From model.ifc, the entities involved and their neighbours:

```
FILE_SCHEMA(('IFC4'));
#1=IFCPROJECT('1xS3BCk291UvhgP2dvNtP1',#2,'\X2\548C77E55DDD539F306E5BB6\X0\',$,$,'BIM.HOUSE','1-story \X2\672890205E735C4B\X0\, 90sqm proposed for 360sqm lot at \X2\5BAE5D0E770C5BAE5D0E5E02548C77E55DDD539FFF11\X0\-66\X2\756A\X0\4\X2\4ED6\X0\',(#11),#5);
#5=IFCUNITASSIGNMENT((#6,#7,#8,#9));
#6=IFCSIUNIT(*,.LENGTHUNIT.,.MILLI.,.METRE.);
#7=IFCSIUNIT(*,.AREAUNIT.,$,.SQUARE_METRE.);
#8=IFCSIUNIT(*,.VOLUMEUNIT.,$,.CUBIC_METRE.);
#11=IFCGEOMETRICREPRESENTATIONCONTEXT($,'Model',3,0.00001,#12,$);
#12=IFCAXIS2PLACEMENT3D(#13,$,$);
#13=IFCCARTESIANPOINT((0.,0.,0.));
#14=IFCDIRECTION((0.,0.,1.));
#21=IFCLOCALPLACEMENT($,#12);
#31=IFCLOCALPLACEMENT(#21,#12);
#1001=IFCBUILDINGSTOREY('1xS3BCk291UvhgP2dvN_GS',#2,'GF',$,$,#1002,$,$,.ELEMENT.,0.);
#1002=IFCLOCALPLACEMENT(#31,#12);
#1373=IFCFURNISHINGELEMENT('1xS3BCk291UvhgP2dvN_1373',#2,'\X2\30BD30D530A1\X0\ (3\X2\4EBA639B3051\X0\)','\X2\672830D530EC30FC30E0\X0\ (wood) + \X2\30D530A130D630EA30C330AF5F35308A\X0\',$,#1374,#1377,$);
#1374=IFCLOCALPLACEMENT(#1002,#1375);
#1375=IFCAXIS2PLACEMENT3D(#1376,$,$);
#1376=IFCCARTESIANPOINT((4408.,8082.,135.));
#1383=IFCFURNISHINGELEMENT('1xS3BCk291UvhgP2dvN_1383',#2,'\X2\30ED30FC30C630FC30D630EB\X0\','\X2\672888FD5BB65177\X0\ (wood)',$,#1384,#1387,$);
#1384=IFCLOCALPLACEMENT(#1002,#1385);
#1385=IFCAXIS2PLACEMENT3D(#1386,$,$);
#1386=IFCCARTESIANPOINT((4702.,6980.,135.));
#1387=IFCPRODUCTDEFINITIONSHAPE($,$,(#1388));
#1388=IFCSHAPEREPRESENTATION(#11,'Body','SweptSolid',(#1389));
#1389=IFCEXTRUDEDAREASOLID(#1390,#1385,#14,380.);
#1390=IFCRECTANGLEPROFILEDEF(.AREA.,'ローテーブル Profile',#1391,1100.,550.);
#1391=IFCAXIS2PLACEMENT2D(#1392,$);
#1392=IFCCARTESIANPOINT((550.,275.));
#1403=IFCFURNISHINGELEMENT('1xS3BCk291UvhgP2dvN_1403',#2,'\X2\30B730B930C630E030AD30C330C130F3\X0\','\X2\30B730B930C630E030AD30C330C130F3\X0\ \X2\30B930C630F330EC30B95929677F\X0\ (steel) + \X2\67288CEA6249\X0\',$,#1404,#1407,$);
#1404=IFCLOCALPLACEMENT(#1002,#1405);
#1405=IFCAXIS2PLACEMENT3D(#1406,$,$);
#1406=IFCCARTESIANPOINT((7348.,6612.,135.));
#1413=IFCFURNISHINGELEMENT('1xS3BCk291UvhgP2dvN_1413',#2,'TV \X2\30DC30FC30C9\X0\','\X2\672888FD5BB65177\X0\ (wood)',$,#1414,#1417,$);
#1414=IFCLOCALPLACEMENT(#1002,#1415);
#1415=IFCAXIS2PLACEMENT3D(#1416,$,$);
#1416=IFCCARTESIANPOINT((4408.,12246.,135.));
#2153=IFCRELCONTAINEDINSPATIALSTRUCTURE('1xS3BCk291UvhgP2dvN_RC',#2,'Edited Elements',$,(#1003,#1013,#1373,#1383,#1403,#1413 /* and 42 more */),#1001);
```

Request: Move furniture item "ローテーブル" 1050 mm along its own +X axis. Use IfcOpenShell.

```python
import ifcopenshell
import ifcopenshell.api.geometry
import ifcopenshell.util.placement
import ifcopenshell.util.unit

model = ifcopenshell.open("model.ifc")
unit_scale = ifcopenshell.util.unit.calculate_unit_scale(model)

item = model.by_id(1383)
matrix = ifcopenshell.util.placement.get_local_placement(item.ObjectPlacement)
matrix[:3, 3] += matrix[:3, 0] * 1.05 / unit_scale
ifcopenshell.api.geometry.edit_object_placement(model, product=item, matrix=matrix, is_si=False)

print(ifcopenshell.util.placement.get_local_placement(item.ObjectPlacement).round(3) + 0.0)

model.write("model_edited.ifc")
```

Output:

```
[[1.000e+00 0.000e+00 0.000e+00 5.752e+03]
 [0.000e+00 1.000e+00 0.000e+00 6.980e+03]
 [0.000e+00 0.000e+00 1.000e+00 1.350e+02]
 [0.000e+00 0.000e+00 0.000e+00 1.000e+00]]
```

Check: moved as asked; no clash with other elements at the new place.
